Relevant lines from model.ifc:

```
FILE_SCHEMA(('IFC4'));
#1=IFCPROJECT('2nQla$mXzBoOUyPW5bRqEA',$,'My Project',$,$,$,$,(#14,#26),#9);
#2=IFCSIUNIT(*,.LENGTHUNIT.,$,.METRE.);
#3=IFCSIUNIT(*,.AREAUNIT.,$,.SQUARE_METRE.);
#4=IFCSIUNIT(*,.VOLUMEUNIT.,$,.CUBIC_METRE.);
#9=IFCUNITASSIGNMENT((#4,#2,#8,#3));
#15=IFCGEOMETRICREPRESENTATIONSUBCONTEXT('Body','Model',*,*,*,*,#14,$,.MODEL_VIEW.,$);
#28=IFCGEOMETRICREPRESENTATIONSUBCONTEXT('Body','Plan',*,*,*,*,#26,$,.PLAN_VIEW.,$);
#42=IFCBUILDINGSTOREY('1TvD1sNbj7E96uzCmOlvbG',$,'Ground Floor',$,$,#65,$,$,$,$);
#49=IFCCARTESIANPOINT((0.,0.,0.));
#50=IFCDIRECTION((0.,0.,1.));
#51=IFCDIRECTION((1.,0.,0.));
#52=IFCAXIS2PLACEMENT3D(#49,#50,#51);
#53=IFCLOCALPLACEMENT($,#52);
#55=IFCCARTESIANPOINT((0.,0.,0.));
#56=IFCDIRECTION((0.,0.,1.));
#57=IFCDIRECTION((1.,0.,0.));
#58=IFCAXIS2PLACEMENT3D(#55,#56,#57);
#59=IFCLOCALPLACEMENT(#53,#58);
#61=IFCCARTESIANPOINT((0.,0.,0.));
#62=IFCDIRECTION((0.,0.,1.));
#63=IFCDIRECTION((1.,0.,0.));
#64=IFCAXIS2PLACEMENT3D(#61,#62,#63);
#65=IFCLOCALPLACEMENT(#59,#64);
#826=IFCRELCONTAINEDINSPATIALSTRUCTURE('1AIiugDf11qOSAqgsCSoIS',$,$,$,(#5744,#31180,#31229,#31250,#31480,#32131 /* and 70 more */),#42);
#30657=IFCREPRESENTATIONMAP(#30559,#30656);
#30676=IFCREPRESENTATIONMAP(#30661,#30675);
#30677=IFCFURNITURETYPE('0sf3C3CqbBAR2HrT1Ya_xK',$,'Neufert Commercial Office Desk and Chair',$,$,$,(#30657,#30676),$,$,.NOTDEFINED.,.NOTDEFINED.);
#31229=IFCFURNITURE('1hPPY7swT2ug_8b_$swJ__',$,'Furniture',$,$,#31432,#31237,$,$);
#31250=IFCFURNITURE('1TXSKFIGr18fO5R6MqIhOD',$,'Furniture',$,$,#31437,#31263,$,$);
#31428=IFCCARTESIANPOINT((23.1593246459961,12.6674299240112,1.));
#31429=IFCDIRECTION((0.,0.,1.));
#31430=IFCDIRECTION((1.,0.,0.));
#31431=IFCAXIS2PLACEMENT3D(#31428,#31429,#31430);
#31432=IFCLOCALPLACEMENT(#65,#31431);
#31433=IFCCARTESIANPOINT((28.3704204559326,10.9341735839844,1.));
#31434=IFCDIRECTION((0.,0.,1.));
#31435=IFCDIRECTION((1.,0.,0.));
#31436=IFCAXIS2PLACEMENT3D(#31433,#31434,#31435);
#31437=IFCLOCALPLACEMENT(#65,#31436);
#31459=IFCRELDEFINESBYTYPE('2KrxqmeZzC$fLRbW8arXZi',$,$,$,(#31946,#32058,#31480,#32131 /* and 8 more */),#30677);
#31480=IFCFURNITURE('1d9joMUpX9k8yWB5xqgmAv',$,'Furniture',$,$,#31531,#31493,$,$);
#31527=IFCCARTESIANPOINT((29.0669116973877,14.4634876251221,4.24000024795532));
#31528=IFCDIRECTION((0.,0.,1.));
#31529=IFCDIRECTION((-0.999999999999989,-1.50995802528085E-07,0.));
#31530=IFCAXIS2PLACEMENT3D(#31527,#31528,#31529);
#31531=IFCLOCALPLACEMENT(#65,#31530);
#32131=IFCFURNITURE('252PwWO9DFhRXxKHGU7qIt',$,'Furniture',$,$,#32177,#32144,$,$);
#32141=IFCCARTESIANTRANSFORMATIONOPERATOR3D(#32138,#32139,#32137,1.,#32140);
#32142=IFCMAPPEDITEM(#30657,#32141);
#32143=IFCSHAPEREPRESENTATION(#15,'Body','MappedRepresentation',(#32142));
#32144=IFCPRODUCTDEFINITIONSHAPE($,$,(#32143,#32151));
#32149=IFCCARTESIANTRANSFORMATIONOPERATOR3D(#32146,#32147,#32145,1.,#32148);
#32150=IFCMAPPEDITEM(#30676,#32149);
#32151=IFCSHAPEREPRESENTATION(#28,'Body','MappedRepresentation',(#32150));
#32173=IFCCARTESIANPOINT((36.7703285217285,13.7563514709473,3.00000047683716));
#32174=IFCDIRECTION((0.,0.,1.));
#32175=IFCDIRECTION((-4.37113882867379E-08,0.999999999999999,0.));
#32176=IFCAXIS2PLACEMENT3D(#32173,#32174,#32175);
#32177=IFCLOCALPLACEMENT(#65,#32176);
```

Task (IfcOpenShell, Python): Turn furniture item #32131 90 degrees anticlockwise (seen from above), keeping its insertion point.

```python
import ifcopenshell
import ifcopenshell.api.geometry
import ifcopenshell.util.placement

model = ifcopenshell.open("model.ifc")

item = model.by_id(32131)
matrix = ifcopenshell.util.placement.get_local_placement(item.ObjectPlacement)
matrix = matrix @ ifcopenshell.util.placement.rotation(90, "Z")
ifcopenshell.api.geometry.edit_object_placement(model, product=item, matrix=matrix, is_si=False)

print(ifcopenshell.util.placement.get_local_placement(item.ObjectPlacement).round(3) + 0.0)

model.write("model_rev.ifc")
```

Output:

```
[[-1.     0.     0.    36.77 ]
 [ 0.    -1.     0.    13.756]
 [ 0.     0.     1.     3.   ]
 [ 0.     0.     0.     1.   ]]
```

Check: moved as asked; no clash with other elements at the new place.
